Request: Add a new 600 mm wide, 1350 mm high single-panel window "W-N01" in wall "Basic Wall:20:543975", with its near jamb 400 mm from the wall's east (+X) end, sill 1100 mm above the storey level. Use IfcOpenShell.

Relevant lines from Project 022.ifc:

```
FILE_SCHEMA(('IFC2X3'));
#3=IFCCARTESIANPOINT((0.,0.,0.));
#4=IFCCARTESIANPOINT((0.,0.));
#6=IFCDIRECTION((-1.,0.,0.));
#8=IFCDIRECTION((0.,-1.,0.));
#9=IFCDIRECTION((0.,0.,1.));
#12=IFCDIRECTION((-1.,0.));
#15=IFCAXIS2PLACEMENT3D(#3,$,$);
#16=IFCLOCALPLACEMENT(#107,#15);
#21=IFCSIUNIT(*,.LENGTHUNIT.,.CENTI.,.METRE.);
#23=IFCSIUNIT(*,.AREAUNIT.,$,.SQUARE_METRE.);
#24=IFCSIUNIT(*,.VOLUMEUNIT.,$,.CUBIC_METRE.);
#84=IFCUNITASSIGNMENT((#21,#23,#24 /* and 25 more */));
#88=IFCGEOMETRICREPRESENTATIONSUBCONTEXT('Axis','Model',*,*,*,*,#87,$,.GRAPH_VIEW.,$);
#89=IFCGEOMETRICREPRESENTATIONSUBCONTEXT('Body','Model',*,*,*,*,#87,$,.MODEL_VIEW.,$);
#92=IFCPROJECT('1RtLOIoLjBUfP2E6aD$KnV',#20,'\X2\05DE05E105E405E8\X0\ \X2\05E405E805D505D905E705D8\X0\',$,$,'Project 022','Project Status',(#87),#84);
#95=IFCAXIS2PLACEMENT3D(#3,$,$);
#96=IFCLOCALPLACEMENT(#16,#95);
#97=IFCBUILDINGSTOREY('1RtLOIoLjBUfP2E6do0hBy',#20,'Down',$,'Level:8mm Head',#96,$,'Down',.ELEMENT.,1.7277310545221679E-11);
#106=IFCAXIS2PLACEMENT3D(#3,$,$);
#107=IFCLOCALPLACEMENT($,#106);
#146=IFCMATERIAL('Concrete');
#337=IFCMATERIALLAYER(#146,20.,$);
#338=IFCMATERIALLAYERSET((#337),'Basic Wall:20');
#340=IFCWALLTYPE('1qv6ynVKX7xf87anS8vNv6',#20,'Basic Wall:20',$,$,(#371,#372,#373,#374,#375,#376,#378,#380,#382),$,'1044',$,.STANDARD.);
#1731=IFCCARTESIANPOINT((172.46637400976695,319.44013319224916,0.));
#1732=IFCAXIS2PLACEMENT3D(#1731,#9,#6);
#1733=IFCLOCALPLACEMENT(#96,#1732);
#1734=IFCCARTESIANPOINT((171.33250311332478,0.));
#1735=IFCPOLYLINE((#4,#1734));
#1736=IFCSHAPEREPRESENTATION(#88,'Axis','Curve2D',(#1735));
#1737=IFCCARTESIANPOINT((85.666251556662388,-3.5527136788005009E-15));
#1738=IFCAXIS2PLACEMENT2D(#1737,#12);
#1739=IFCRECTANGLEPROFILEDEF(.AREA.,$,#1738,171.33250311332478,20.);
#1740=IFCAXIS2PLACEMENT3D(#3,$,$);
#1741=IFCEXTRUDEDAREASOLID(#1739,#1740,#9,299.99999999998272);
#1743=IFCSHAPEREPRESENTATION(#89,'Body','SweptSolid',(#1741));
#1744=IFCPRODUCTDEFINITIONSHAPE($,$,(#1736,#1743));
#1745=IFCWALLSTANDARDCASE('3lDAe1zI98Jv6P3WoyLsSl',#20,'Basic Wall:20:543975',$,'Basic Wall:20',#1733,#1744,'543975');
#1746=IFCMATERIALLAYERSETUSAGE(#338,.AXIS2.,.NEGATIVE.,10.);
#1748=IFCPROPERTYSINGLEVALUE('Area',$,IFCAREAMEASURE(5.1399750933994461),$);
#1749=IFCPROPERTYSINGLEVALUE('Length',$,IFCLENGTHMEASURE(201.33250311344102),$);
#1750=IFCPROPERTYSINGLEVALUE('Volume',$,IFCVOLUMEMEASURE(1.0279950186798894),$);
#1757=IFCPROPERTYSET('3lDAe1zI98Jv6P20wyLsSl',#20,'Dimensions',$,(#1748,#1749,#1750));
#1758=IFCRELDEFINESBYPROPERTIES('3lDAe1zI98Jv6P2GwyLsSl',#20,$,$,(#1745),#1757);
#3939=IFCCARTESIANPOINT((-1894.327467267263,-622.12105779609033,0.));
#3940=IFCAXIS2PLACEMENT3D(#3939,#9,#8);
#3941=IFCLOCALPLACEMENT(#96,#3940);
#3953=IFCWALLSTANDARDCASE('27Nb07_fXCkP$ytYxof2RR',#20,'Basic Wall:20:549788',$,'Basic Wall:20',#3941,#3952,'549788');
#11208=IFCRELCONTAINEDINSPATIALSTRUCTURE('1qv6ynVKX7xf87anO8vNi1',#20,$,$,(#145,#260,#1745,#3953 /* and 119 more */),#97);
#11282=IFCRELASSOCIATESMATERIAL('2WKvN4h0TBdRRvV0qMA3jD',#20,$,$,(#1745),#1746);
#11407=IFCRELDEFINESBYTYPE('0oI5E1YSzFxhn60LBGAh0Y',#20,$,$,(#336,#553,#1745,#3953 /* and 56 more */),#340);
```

```python
import numpy as np
import ifcopenshell
import ifcopenshell.api.feature
import ifcopenshell.api.geometry
import ifcopenshell.api.pset
import ifcopenshell.api.root
import ifcopenshell.api.spatial
import ifcopenshell.api.type
import ifcopenshell.geom
import ifcopenshell.util.element
import ifcopenshell.util.placement
import ifcopenshell.util.representation
import ifcopenshell.util.shape
import ifcopenshell.util.unit

model = ifcopenshell.open("Project 022.ifc")
unit_scale = ifcopenshell.util.unit.calculate_unit_scale(model)
area_scale = ifcopenshell.util.unit.calculate_unit_scale(model, "AREAUNIT")
volume_scale = ifcopenshell.util.unit.calculate_unit_scale(model, "VOLUMEUNIT")
settings = ifcopenshell.geom.settings()


def volume(element):
    """Net volume in cubic metres, openings subtracted."""
    shape = ifcopenshell.geom.create_shape(settings, element)
    return ifcopenshell.util.shape.get_volume(shape.geometry)


wall = model.by_id(1745)
storey = ifcopenshell.util.element.get_container(wall, ifc_class="IfcBuildingStorey")
context = ifcopenshell.util.representation.get_context(model, "Model", "Body", "MODEL_VIEW")
before = volume(wall)

width, height, from_end, sill = 0.6, 1.35, 0.4, 1.1  # metres

# The wall runs along its own X axis, and the end named is its -X end.
wall_shape = ifcopenshell.geom.create_shape(settings, wall)
x, y, z = ifcopenshell.util.shape.get_vertices(wall_shape.geometry).T
start = x.min() + from_end
face, thickness = float(y.min()), float(y.max() - y.min())
wall_matrix = ifcopenshell.util.placement.get_local_placement(wall.ObjectPlacement)
level = ifcopenshell.util.placement.get_local_placement(storey.ObjectPlacement)[2, 3]


def in_wall(x, y):
    """Placement at x, y metres in the wall's axes, at sill height."""
    matrix = wall_matrix.copy()
    matrix[:, 3] = wall_matrix @ np.array([x / unit_scale, y / unit_scale, 0.0, 1.0])
    matrix[2, 3] = level + sill / unit_scale
    return matrix


# Opening: a box that overshoots both wall faces by 50 mm.
opening = ifcopenshell.api.root.create_entity(model, ifc_class="IfcOpeningElement")
box = ifcopenshell.api.geometry.add_wall_representation(
    model, context=context, length=width, height=height, thickness=thickness + 0.1
)
ifcopenshell.api.geometry.assign_representation(model, product=opening, representation=box)
ifcopenshell.api.geometry.edit_object_placement(model, product=opening, matrix=in_wall(start, face - 0.05), is_si=False)
ifcopenshell.api.feature.add_feature(model, feature=opening, element=wall)

window = ifcopenshell.api.root.create_entity(model, ifc_class="IfcWindow", name="W-N01")
window.OverallWidth, window.OverallHeight = width / unit_scale, height / unit_scale
body = ifcopenshell.api.geometry.add_window_representation(
    model,
    context=context,
    overall_width=window.OverallWidth,
    overall_height=window.OverallHeight,
    partition_type="SINGLE_PANEL",
)
ifcopenshell.api.geometry.assign_representation(model, product=window, representation=body)
ifcopenshell.api.spatial.assign_container(model, products=[window], relating_structure=storey)
fills = ifcopenshell.api.feature.add_filling(model, opening=opening, element=window)
fills.OwnerHistory = window.OwnerHistory  # required in IFC2X3

# IFC2X3 keeps the operation on the window style.
style = ifcopenshell.api.root.create_entity(model, ifc_class="IfcWindowStyle", name="W-N01")
style.OperationType, style.ConstructionType = "SINGLE_PANEL", "NOTDEFINED"
style.ParameterTakesPrecedence = style.Sizeable = False
ifcopenshell.api.type.assign_type(model, related_objects=[window], relating_type=style)

# Centre the window in the wall's thickness.
ifcopenshell.api.geometry.edit_object_placement(model, product=window, matrix=in_wall(start, face), is_si=False)
window_shape = ifcopenshell.geom.create_shape(settings, window)
depth = ifcopenshell.util.shape.get_vertices(window_shape.geometry)[:, 1]
offset = face + thickness / 2 - (depth.min() + depth.max()) / 2
ifcopenshell.api.geometry.edit_object_placement(model, product=window, matrix=in_wall(start, offset), is_si=False)

after = volume(wall)

# Update the wall's stored quantities.
pset = model.by_id(ifcopenshell.util.element.get_pset(wall, "Dimensions", should_inherit=False)["id"])
ifcopenshell.api.pset.edit_pset(model, pset=pset, properties={
    "Area": model.create_entity("IfcAreaMeasure", after / thickness / area_scale),
    "Volume": model.create_entity("IfcVolumeMeasure", after / volume_scale),
})

print(f"wall volume {before:.3f} -> {after:.3f} m3")

model.write("Project 022_updated.ifc")
```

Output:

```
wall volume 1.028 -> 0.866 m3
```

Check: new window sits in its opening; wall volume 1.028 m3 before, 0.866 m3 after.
